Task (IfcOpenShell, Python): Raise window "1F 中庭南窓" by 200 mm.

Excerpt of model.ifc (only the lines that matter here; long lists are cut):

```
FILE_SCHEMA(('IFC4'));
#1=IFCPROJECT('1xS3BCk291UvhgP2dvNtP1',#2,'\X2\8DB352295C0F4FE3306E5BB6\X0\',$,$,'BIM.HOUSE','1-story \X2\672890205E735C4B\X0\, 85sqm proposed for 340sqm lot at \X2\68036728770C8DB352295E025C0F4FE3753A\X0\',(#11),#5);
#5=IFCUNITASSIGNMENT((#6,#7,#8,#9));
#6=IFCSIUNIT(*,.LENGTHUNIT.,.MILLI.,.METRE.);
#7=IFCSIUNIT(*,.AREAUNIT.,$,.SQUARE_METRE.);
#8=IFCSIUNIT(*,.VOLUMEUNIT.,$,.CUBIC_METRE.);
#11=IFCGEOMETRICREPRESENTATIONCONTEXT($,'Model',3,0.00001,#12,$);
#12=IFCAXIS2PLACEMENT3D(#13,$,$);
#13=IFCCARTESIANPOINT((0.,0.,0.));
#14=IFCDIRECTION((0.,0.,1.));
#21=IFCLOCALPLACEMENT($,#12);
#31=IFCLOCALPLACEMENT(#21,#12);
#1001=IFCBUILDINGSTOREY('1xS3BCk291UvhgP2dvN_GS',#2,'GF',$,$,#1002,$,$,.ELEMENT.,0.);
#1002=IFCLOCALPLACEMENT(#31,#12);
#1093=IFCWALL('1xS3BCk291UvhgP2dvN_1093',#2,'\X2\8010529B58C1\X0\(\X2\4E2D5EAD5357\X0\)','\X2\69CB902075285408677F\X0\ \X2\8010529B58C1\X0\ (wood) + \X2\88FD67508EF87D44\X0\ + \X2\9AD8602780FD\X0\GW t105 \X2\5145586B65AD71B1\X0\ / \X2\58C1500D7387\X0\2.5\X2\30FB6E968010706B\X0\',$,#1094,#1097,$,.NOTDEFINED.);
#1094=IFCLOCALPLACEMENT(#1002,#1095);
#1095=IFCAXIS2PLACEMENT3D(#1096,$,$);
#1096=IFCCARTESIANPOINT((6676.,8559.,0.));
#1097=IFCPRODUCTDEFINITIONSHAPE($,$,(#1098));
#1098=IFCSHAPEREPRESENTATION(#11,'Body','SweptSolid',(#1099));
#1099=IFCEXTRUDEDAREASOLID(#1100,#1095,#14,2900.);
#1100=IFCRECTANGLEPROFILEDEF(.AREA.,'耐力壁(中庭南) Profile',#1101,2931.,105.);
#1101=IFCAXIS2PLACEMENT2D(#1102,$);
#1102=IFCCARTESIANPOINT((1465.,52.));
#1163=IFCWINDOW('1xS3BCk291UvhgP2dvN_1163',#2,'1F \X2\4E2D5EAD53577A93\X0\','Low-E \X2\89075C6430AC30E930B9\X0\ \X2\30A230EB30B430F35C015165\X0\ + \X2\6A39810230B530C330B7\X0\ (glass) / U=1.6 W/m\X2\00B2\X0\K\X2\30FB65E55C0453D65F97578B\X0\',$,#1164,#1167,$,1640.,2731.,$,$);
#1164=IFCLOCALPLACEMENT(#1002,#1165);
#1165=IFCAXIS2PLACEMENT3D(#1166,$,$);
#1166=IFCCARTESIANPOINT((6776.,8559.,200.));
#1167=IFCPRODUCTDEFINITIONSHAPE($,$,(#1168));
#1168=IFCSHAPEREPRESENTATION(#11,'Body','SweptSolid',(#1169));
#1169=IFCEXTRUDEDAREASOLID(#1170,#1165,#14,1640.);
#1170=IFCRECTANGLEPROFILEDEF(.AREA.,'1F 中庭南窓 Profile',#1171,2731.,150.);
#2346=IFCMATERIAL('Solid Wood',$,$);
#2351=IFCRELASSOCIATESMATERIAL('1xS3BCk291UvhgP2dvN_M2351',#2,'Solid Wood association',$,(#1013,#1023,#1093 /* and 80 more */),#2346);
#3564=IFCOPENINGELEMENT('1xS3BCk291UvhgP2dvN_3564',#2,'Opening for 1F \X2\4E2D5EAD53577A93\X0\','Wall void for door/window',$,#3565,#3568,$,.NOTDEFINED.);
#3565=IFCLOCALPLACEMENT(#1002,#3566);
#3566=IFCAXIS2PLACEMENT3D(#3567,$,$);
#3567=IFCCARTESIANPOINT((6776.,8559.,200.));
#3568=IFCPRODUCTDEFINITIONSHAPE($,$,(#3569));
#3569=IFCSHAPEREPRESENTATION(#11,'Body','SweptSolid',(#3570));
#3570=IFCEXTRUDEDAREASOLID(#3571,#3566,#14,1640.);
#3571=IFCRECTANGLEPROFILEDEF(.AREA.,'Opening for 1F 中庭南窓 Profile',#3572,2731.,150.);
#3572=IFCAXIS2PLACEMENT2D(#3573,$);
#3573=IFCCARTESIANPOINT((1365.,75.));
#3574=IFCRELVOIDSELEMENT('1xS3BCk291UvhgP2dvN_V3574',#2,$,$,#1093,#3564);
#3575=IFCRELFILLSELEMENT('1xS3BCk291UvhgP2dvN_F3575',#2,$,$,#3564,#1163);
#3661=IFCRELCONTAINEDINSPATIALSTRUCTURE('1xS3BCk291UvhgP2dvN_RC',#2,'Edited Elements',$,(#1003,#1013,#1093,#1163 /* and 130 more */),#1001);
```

```python
import numpy as np
import ifcopenshell
import ifcopenshell.api.geometry
import ifcopenshell.util.placement
import ifcopenshell.util.unit

model = ifcopenshell.open("model.ifc")
unit_scale = ifcopenshell.util.unit.calculate_unit_scale(model)

window = model.by_guid("1xS3BCk291UvhgP2dvN_1163")
opening = window.FillsVoids[0].RelatingOpeningElement
dz = 200.0

shift = np.array([0.0, 0.0, dz])
# The window is not placed relative to its opening, so move both.
for product in (opening, window):
    matrix = ifcopenshell.util.placement.get_local_placement(product.ObjectPlacement)
    matrix[:3, 3] += shift
    ifcopenshell.api.geometry.edit_object_placement(model, product=product, matrix=matrix, is_si=False)

print(f"moved by {dz * unit_scale:+.3f} m")

model.write("model-out.ifc")
```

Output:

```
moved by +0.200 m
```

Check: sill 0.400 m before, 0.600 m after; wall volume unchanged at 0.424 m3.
